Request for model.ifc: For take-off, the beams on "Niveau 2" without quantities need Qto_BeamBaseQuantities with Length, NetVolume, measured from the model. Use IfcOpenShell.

First a look at what the model holds.

```python
import ifcopenshell
import ifcopenshell.util.element
import ifcopenshell.util.unit

model = ifcopenshell.open("model.ifc")
print(model.schema)
for unit_type in ("LENGTHUNIT", "AREAUNIT", "VOLUMEUNIT"):
    print(unit_type, ifcopenshell.util.unit.calculate_unit_scale(model, unit_type))
storey = next(s for s in model.by_type("IfcBuildingStorey") if s.Name == "Niveau 2")
beams = [e for e in ifcopenshell.util.element.get_decomposition(storey) if e.is_a("IfcBeam")]
for e in sorted(beams, key=lambda e: e.id()):
    print(e.id(), e.is_a(), e.Name, list(ifcopenshell.util.element.get_psets(e, qtos_only=True)), sep=" | ")
```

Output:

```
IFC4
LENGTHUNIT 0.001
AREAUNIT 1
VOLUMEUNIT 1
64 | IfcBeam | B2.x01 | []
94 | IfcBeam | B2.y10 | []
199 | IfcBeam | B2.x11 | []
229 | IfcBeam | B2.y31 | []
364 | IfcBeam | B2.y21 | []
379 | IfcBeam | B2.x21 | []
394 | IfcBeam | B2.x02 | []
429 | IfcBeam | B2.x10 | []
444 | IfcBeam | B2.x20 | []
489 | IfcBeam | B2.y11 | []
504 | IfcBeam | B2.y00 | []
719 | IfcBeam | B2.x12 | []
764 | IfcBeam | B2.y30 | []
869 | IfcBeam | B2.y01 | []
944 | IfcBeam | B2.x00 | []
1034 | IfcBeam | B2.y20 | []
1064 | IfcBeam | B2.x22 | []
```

```python
import ifcopenshell
import ifcopenshell.api.pset
import ifcopenshell.geom
import ifcopenshell.util.element
import ifcopenshell.util.shape
import ifcopenshell.util.unit

model = ifcopenshell.open("model.ifc")
unit_scale = ifcopenshell.util.unit.calculate_unit_scale(model)
volume_scale = ifcopenshell.util.unit.calculate_unit_scale(model, "VOLUMEUNIT")
settings = ifcopenshell.geom.settings()

storey = next(s for s in model.by_type("IfcBuildingStorey") if s.Name == "Niveau 2")
beams = [e for e in ifcopenshell.util.element.get_decomposition(storey) if e.is_a("IfcBeam")]

for e in sorted(beams, key=lambda e: e.id()):
    if ifcopenshell.util.element.get_psets(e, qtos_only=True, should_inherit=False):
        continue
    # Geometry comes back in metres, in the element's own axes.
    shape = ifcopenshell.geom.create_shape(settings, e)
    values = {
        "Length": ifcopenshell.util.shape.get_max_xyz(shape.geometry) / unit_scale,
        "NetVolume": ifcopenshell.util.shape.get_volume(shape.geometry) / volume_scale,
    }
    qto = ifcopenshell.api.pset.add_qto(model, product=e, name="Qto_BeamBaseQuantities")
    ifcopenshell.api.pset.edit_qto(model, qto=qto, properties=values)
    print(e.id(), {k: round(v, 3) for k, v in values.items()})

model.write("model_edited.ifc")
```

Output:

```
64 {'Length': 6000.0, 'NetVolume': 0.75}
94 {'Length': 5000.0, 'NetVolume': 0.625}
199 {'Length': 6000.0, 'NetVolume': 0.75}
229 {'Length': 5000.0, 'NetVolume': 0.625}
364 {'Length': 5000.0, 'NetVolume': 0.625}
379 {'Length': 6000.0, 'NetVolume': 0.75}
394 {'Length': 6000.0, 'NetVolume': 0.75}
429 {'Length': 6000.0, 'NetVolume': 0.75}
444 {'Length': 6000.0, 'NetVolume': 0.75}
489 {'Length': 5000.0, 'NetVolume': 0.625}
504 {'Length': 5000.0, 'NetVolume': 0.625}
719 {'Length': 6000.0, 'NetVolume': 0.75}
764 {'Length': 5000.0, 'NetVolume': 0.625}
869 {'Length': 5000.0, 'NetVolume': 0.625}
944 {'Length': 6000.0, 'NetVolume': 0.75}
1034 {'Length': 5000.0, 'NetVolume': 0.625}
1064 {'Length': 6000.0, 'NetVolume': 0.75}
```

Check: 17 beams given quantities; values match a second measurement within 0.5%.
